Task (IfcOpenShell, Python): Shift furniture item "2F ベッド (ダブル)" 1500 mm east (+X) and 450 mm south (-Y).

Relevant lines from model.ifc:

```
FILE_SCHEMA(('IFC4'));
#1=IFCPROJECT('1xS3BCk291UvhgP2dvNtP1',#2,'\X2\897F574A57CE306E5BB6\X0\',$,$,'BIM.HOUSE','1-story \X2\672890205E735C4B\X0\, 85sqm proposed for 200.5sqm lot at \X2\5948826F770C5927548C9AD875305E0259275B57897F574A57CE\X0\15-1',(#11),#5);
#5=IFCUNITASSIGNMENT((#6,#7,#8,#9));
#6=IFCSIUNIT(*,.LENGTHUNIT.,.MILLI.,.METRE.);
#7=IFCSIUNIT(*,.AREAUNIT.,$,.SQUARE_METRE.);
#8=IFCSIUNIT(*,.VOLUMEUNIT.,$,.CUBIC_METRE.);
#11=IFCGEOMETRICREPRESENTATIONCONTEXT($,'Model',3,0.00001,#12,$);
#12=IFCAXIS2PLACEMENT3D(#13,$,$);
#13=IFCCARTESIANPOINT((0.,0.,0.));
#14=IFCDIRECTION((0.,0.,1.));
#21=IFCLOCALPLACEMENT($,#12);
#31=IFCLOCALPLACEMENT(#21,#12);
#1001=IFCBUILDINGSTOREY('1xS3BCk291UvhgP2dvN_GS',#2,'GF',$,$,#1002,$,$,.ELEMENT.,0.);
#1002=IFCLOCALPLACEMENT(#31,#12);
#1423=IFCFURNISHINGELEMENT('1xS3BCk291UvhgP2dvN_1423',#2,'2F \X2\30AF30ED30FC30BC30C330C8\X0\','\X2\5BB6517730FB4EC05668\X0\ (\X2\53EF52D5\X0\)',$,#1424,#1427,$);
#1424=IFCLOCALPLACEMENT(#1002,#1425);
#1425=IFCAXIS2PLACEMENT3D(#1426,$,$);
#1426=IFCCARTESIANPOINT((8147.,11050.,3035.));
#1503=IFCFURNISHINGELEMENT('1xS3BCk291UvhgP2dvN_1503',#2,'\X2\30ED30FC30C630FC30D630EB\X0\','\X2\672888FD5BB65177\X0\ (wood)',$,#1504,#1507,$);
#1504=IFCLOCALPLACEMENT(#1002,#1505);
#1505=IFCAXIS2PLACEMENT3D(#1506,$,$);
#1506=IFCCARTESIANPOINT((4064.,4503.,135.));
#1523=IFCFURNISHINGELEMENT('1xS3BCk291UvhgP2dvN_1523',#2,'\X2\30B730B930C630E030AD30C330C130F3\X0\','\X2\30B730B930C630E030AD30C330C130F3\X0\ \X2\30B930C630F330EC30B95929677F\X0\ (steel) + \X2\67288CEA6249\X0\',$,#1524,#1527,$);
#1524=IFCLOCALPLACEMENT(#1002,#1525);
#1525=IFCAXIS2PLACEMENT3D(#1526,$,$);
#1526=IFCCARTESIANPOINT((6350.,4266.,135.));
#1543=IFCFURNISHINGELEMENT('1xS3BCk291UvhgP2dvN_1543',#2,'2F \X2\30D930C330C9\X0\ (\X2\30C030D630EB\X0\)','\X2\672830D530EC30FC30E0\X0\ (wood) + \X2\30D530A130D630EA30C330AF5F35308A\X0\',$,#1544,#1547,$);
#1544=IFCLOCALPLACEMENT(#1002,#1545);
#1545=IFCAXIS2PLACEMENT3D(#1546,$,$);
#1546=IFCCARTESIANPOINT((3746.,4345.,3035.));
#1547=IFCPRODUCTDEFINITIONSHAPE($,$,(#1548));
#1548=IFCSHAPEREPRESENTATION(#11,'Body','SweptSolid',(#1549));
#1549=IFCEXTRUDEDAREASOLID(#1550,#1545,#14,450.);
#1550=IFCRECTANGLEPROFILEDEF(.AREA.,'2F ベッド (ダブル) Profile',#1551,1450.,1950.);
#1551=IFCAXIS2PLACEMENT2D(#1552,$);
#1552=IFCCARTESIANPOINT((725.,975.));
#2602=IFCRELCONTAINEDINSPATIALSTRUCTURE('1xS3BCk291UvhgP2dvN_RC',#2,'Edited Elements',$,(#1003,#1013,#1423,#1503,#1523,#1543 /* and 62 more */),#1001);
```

```python
import ifcopenshell
import ifcopenshell.api.geometry
import ifcopenshell.util.placement
import ifcopenshell.util.unit

model = ifcopenshell.open("model.ifc")
unit_scale = ifcopenshell.util.unit.calculate_unit_scale(model)

item = model.by_guid("1xS3BCk291UvhgP2dvN_1543")
matrix = ifcopenshell.util.placement.get_local_placement(item.ObjectPlacement)
matrix[0, 3] += 1.5 / unit_scale
matrix[1, 3] -= 0.45 / unit_scale
ifcopenshell.api.geometry.edit_object_placement(model, product=item, matrix=matrix, is_si=False)

print(ifcopenshell.util.placement.get_local_placement(item.ObjectPlacement).round(3) + 0.0)

model.write("model_v2.ifc")
```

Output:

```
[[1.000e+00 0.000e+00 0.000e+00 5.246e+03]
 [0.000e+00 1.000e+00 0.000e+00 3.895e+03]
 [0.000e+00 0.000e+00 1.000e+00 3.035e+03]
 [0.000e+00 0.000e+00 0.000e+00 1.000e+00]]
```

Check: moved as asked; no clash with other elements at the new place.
